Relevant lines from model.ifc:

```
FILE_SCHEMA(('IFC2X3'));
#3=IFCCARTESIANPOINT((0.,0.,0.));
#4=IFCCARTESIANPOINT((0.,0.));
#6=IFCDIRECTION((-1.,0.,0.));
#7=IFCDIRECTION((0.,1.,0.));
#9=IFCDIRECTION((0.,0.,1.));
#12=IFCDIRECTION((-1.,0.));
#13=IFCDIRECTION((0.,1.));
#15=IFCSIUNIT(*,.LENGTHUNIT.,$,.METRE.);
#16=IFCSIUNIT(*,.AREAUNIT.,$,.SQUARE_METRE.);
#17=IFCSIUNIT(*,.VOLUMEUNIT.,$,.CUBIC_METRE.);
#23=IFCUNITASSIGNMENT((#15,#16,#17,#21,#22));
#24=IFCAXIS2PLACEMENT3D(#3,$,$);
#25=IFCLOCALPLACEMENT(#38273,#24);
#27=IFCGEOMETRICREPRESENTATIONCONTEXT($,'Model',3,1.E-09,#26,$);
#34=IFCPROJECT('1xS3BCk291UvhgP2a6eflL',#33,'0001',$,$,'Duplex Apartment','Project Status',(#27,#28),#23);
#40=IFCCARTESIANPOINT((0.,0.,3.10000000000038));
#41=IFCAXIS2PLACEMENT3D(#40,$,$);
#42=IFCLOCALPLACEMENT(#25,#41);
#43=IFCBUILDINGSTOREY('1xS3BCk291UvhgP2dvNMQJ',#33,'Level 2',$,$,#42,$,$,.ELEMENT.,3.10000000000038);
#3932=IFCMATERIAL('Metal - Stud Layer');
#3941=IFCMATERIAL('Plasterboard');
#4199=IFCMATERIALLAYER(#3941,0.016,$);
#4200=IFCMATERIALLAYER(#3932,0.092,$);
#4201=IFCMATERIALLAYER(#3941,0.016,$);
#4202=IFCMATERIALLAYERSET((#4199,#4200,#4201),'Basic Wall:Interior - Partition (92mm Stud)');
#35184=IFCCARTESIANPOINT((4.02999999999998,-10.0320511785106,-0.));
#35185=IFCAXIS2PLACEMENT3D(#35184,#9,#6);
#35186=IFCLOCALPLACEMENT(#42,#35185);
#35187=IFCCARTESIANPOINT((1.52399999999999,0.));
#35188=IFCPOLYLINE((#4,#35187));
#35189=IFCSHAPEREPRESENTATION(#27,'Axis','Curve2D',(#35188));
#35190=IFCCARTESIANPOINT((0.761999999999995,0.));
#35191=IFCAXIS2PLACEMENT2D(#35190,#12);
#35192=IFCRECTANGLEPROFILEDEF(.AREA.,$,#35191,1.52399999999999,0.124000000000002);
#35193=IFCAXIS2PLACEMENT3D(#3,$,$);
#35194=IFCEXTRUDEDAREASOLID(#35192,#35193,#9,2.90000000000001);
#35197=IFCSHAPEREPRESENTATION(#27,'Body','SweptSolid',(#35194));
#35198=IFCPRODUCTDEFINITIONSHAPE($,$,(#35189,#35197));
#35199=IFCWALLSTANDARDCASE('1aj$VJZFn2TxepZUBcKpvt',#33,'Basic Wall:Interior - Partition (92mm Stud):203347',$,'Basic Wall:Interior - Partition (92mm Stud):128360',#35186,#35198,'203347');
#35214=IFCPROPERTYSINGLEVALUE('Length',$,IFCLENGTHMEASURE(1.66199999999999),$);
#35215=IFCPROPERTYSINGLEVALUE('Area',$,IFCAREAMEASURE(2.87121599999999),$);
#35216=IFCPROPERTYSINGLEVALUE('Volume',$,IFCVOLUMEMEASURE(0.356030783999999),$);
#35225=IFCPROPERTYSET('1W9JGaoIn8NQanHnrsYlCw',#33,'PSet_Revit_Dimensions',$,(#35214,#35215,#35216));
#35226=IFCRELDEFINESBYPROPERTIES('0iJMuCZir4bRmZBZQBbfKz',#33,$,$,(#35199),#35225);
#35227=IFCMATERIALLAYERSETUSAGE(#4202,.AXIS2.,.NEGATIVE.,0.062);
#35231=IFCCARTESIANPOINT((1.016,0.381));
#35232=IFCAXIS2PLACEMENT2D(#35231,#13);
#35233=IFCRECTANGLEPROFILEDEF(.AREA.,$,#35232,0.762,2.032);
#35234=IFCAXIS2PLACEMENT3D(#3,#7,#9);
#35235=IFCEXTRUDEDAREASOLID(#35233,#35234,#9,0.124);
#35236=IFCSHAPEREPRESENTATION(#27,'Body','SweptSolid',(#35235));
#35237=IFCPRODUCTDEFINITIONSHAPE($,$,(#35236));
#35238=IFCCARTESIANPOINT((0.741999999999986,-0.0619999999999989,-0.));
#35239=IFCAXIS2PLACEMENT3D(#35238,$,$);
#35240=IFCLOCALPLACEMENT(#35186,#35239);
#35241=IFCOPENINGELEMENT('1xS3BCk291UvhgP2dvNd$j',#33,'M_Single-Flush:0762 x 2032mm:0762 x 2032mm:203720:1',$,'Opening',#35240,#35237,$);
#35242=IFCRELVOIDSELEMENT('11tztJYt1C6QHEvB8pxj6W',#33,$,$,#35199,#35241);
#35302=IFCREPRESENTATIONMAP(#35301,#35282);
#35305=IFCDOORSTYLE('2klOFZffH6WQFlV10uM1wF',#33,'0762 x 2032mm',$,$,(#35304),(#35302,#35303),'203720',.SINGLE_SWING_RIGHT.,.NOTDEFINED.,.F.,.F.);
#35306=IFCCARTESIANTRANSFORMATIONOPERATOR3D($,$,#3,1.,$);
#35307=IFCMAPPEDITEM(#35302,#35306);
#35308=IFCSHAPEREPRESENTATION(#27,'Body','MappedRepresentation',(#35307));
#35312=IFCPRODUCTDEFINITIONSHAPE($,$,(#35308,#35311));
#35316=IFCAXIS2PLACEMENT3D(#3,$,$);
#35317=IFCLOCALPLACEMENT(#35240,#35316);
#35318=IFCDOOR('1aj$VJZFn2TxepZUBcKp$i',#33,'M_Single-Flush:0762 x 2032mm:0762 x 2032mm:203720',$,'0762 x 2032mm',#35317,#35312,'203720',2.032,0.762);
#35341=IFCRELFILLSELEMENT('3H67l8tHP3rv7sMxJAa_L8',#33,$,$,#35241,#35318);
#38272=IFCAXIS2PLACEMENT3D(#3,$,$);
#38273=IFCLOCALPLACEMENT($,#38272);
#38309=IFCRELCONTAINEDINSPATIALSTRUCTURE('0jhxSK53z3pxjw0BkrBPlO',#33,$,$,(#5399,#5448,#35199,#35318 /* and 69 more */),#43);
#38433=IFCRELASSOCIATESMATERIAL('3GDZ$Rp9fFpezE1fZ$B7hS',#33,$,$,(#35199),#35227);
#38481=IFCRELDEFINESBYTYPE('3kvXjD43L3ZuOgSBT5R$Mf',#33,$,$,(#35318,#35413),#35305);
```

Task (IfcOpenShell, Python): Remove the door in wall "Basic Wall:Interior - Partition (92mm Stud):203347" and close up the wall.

```python
import ifcopenshell
import ifcopenshell.api.feature
import ifcopenshell.api.pset
import ifcopenshell.api.root
import ifcopenshell.geom
import ifcopenshell.util.element
import ifcopenshell.util.shape
import ifcopenshell.util.unit

model = ifcopenshell.open("model.ifc")
area_scale = ifcopenshell.util.unit.calculate_unit_scale(model, "AREAUNIT")
volume_scale = ifcopenshell.util.unit.calculate_unit_scale(model, "VOLUMEUNIT")
settings = ifcopenshell.geom.settings()


def volume(element):
    """Net volume in cubic metres, openings subtracted."""
    shape = ifcopenshell.geom.create_shape(settings, element)
    return ifcopenshell.util.shape.get_volume(shape.geometry)


door = model.by_guid("1aj$VJZFn2TxepZUBcKp$i")
opening = door.FillsVoids[0].RelatingOpeningElement
wall = opening.VoidsElements[0].RelatingBuildingElement
before = volume(wall)

ifcopenshell.api.root.remove_product(model, product=door)
ifcopenshell.api.feature.remove_feature(model, feature=opening)

after = volume(wall)
thickness = 0.124  # wall thickness in metres

# Update the wall's stored quantities.
pset = model.by_id(ifcopenshell.util.element.get_pset(wall, "PSet_Revit_Dimensions", should_inherit=False)["id"])
ifcopenshell.api.pset.edit_pset(model, pset=pset, properties={
    "Area": model.create_entity("IfcAreaMeasure", after / thickness / area_scale),
    "Volume": model.create_entity("IfcVolumeMeasure", after / volume_scale),
})

print(f"wall volume {before:.3f} -> {after:.3f} m3")

model.write("model_updated.ifc")
```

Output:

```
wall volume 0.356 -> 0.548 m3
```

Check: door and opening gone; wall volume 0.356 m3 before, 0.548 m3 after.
